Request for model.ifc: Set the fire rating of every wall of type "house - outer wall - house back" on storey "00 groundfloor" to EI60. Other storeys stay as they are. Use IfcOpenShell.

First a look at what the model holds.

```python
import ifcopenshell
import ifcopenshell.util.element

model = ifcopenshell.open("model.ifc")
print(model.schema)
storey = next(s for s in model.by_type("IfcBuildingStorey") if s.Name == "00 groundfloor")
walls = [e for e in ifcopenshell.util.element.get_decomposition(storey) if e.is_a("IfcWall")]
seen = {}
for e in walls:
    element_type = ifcopenshell.util.element.get_type(e)
    key = (element_type.Name if element_type != e and element_type else None, ifcopenshell.util.element.get_pset(e, "Pset_WallCommon", "FireRating"))
    seen[key] = seen.get(key, 0) + 1
for (name, value), count in sorted(seen.items(), key=str):
    print(count, "x", name, "|", value)
```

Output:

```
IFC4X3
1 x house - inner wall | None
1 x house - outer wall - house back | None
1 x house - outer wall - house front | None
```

```python
import ifcopenshell
import ifcopenshell.api.pset
import ifcopenshell.util.element

model = ifcopenshell.open("model.ifc")

storey = next(s for s in model.by_type("IfcBuildingStorey") if s.Name == "00 groundfloor")
walls = [e for e in ifcopenshell.util.element.get_decomposition(storey) if e.is_a("IfcWall")]

count = 0
for e in walls:
    element_type = ifcopenshell.util.element.get_type(e)
    if element_type in (None, e) or element_type.Name != "house - outer wall - house back":
        continue
    # add_pset returns the element's existing set when there is one.
    pset = ifcopenshell.api.pset.add_pset(model, product=e, name="Pset_WallCommon")
    ifcopenshell.api.pset.edit_pset(model, pset=pset, properties={"FireRating": "EI60"})
    count += 1

print(count, "walls updated")

model.write("model_rev.ifc")
```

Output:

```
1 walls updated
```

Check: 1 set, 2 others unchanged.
